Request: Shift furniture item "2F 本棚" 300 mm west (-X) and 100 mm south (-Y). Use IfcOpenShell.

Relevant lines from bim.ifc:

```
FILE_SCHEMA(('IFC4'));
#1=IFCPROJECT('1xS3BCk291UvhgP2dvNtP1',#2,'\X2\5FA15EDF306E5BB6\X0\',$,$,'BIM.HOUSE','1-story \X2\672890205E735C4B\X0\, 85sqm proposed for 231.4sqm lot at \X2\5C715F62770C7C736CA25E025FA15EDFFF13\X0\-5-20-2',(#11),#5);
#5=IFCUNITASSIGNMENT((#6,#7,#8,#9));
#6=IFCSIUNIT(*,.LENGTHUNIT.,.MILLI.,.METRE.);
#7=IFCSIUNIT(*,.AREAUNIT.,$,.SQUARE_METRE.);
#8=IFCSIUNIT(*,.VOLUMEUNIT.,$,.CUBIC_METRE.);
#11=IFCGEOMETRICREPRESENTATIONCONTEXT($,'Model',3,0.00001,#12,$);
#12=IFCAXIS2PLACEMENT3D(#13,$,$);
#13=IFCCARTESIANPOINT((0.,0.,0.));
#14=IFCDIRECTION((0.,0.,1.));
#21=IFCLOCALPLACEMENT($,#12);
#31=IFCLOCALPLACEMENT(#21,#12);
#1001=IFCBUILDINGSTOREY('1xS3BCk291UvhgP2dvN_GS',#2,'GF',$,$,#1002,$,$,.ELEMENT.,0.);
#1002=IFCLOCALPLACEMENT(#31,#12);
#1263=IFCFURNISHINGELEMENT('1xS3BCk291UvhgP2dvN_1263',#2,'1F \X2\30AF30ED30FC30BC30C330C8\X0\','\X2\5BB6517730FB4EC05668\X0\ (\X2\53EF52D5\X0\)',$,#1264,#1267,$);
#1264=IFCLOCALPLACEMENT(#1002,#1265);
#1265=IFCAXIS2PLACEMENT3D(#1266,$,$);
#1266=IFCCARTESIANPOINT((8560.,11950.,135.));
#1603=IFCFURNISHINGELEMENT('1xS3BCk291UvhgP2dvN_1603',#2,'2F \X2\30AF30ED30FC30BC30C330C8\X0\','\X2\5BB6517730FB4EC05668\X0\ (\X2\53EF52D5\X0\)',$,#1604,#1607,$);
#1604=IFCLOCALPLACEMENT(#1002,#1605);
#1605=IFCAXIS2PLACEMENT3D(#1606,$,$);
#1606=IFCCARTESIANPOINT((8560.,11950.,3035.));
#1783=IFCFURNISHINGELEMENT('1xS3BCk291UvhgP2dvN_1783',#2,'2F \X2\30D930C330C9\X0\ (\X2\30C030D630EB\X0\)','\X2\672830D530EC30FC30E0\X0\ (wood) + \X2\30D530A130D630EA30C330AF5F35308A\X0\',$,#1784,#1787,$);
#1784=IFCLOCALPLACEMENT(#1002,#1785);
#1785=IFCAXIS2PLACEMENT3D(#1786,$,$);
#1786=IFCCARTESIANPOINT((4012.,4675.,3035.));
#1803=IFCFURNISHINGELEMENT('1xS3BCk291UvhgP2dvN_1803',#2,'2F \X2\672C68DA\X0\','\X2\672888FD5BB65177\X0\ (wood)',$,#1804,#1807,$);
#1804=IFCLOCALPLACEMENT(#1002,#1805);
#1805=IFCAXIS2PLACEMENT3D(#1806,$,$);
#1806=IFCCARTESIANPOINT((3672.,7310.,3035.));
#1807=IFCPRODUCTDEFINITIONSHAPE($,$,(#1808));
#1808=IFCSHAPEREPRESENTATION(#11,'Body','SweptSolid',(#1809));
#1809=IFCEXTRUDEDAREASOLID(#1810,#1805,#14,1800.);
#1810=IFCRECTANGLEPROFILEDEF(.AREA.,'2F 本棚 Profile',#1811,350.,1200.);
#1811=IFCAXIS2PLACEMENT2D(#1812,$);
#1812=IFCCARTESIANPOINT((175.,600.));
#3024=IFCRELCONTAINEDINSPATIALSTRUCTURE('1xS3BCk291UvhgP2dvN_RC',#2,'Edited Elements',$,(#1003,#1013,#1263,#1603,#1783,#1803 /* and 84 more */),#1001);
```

```python
import ifcopenshell
import ifcopenshell.api.geometry
import ifcopenshell.util.placement

model = ifcopenshell.open("bim.ifc")

item = model.by_guid("1xS3BCk291UvhgP2dvN_1803")
matrix = ifcopenshell.util.placement.get_local_placement(item.ObjectPlacement)
matrix[0, 3] -= 300.0
matrix[1, 3] -= 100.0
ifcopenshell.api.geometry.edit_object_placement(model, product=item, matrix=matrix, is_si=False)

print(ifcopenshell.util.placement.get_local_placement(item.ObjectPlacement).round(3) + 0.0)

model.write("bim-out.ifc")
```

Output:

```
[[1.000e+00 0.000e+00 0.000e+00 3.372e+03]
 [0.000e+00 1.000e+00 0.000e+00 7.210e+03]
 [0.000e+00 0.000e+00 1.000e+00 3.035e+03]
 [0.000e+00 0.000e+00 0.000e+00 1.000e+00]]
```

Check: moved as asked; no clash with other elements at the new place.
